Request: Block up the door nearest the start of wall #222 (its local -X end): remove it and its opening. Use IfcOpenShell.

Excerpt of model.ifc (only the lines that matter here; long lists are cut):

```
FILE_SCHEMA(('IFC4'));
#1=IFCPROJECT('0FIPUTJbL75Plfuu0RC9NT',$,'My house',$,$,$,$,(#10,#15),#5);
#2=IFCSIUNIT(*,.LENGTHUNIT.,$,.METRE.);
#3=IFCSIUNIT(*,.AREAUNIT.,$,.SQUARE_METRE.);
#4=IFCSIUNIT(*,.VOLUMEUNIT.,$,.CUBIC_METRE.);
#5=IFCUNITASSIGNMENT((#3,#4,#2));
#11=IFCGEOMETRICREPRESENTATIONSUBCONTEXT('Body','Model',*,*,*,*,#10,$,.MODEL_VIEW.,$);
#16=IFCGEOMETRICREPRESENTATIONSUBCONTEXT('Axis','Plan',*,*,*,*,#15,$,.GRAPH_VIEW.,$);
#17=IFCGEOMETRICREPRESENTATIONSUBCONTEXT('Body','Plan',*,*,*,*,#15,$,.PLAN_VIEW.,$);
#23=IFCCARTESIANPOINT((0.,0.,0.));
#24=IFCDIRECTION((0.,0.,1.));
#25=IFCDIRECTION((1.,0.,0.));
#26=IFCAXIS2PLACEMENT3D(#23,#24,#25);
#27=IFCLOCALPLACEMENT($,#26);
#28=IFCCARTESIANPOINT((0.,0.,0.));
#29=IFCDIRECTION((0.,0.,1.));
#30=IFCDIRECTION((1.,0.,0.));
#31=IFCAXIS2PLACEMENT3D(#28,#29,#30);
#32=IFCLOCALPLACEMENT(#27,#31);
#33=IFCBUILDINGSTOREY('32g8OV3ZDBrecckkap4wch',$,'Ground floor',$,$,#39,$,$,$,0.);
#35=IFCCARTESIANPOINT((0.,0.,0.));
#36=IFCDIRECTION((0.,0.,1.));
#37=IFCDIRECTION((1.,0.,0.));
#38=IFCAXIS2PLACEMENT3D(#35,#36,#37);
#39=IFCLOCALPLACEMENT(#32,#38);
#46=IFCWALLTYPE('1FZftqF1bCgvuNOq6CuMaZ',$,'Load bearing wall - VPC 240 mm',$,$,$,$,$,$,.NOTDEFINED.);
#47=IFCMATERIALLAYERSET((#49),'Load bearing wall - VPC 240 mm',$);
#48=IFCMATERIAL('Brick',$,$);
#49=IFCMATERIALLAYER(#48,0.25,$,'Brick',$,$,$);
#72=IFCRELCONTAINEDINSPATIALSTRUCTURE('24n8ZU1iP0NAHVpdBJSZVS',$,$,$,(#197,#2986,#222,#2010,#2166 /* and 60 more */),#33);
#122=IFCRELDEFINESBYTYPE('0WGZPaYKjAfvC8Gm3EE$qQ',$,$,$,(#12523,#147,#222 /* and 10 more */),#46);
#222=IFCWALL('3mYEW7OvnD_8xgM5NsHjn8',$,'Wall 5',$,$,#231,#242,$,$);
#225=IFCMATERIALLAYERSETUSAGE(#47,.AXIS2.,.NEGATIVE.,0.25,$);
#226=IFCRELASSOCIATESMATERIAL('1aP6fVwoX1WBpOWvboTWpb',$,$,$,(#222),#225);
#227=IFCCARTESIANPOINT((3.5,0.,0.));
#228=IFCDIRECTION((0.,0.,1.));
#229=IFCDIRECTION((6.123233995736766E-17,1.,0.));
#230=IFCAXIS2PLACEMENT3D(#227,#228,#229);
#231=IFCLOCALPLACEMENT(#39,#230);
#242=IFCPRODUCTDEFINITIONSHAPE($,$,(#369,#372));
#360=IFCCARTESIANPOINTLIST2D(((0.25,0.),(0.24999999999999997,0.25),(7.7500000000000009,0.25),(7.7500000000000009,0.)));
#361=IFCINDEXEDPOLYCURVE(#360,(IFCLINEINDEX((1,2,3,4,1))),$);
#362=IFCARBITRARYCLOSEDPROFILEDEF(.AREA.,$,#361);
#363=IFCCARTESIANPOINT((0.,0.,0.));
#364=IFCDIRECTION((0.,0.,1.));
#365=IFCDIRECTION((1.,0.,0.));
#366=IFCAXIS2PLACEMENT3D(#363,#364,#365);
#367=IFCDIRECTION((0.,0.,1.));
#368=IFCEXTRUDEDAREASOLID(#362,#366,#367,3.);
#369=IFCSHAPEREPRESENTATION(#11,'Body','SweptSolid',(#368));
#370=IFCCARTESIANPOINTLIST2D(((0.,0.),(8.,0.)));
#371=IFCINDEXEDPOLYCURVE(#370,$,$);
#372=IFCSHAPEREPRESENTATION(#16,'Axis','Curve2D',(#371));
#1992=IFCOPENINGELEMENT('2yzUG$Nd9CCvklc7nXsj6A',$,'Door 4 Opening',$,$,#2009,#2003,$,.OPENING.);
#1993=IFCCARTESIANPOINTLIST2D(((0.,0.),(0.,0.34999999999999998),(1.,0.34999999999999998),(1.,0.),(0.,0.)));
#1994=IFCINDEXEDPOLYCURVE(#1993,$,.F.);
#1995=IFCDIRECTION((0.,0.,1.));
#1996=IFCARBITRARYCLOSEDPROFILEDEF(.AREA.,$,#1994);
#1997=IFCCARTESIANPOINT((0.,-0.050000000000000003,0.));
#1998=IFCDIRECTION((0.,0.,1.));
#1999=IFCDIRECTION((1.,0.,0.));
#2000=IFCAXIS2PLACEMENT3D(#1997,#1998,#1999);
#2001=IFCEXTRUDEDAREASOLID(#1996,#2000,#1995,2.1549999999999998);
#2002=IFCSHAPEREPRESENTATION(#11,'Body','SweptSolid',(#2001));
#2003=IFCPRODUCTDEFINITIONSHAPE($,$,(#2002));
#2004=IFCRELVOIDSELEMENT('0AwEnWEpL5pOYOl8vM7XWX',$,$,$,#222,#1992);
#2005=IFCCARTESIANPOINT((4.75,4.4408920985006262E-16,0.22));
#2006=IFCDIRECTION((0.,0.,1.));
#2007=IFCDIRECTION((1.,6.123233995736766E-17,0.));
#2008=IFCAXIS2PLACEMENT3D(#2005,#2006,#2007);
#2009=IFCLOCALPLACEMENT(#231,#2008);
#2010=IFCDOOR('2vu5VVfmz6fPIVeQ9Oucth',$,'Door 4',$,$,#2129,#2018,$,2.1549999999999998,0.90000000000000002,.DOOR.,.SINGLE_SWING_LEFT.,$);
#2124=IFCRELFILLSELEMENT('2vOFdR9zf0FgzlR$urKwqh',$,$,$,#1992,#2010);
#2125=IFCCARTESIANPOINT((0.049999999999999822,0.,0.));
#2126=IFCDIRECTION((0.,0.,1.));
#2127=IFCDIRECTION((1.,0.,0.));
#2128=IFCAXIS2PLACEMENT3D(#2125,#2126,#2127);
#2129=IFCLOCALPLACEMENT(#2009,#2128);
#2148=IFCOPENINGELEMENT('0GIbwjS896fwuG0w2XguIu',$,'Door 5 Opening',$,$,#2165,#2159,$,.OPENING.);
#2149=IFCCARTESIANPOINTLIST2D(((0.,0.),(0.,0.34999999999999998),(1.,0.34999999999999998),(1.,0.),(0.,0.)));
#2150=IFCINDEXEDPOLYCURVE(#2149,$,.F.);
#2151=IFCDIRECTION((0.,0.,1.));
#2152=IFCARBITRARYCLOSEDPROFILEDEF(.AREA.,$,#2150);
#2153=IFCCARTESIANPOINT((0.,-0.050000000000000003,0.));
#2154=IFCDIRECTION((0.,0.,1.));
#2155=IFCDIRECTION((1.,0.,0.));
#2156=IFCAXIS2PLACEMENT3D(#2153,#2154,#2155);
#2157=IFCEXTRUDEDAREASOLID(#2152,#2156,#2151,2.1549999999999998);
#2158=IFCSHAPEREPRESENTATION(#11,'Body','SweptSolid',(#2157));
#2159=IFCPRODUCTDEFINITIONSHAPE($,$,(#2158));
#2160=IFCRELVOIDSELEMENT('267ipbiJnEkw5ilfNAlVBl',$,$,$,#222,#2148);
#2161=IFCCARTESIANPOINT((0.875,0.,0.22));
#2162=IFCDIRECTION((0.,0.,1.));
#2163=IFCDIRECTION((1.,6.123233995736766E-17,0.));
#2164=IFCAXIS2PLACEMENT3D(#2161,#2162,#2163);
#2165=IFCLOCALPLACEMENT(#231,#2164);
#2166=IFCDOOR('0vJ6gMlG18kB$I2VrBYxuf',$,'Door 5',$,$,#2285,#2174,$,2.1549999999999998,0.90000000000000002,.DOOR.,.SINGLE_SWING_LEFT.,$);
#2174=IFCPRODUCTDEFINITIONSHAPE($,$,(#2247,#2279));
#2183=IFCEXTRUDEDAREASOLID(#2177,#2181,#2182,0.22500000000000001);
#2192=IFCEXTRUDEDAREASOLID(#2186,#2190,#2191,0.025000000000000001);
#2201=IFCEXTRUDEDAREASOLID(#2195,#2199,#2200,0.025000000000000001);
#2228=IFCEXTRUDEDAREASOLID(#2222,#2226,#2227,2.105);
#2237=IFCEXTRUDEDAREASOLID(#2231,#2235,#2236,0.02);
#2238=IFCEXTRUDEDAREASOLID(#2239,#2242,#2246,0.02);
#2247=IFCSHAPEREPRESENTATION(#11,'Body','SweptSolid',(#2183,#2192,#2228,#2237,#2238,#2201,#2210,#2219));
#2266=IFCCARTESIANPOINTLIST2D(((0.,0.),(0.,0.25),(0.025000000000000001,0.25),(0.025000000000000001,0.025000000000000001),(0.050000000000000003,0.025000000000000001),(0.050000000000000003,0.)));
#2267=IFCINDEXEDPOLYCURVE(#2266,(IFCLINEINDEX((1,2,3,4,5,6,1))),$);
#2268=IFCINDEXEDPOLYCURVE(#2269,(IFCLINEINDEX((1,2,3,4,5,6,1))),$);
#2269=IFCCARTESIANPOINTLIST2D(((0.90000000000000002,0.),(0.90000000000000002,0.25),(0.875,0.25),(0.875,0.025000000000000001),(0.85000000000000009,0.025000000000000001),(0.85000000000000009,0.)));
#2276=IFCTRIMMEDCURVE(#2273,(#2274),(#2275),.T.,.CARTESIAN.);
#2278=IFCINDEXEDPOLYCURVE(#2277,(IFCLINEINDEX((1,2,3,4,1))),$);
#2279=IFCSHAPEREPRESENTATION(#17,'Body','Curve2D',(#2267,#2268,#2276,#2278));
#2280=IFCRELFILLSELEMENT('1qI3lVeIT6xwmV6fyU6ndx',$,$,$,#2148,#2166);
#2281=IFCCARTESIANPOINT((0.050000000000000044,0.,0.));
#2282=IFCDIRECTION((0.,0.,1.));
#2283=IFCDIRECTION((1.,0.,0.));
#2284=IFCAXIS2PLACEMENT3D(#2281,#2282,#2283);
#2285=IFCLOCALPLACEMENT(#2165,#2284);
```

```python
import ifcopenshell
import ifcopenshell.api.feature
import ifcopenshell.api.root
import ifcopenshell.geom
import ifcopenshell.util.shape

model = ifcopenshell.open("model.ifc")
settings = ifcopenshell.geom.settings()


def volume(element):
    """Net volume in cubic metres, openings subtracted."""
    shape = ifcopenshell.geom.create_shape(settings, element)
    return ifcopenshell.util.shape.get_volume(shape.geometry)


door = model.by_id(2166)
opening = door.FillsVoids[0].RelatingOpeningElement
wall = opening.VoidsElements[0].RelatingBuildingElement
before = volume(wall)

ifcopenshell.api.root.remove_product(model, product=door)
ifcopenshell.api.feature.remove_feature(model, feature=opening)

after = volume(wall)

print(f"wall volume {before:.3f} -> {after:.3f} m3")

model.write("model_edited.ifc")
```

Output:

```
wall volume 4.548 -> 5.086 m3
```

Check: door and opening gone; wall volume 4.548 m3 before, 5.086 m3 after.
